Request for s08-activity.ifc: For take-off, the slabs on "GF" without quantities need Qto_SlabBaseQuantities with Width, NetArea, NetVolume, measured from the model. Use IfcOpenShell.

First a look at what the model holds.

```python
import ifcopenshell
import ifcopenshell.util.element
import ifcopenshell.util.unit

model = ifcopenshell.open("s08-activity.ifc")
print(model.schema)
for unit_type in ("LENGTHUNIT", "AREAUNIT", "VOLUMEUNIT"):
    print(unit_type, ifcopenshell.util.unit.calculate_unit_scale(model, unit_type))
storey = next(s for s in model.by_type("IfcBuildingStorey") if s.Name == "GF")
slabs = [e for e in ifcopenshell.util.element.get_decomposition(storey) if e.is_a("IfcSlab")]
for e in sorted(slabs, key=lambda e: e.id()):
    print(e.id(), e.is_a(), e.Name, list(ifcopenshell.util.element.get_psets(e, qtos_only=True)), sep=" | ")
```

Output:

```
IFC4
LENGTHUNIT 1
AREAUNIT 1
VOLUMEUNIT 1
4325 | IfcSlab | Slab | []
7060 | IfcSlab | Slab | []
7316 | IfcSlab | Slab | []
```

```python
import ifcopenshell
import ifcopenshell.api.pset
import ifcopenshell.geom
import ifcopenshell.util.element
import ifcopenshell.util.shape
import ifcopenshell.util.unit

model = ifcopenshell.open("s08-activity.ifc")
unit_scale = ifcopenshell.util.unit.calculate_unit_scale(model)
area_scale = ifcopenshell.util.unit.calculate_unit_scale(model, "AREAUNIT")
volume_scale = ifcopenshell.util.unit.calculate_unit_scale(model, "VOLUMEUNIT")
settings = ifcopenshell.geom.settings()

storey = next(s for s in model.by_type("IfcBuildingStorey") if s.Name == "GF")
slabs = [e for e in ifcopenshell.util.element.get_decomposition(storey) if e.is_a("IfcSlab")]

for e in sorted(slabs, key=lambda e: e.id()):
    if ifcopenshell.util.element.get_psets(e, qtos_only=True, should_inherit=False):
        continue
    # Geometry comes back in metres, in the element's own axes.
    shape = ifcopenshell.geom.create_shape(settings, e)
    values = {
        "Width": ifcopenshell.util.shape.get_z(shape.geometry) / unit_scale,
        "NetArea": ifcopenshell.util.shape.get_footprint_area(shape.geometry) / area_scale,
        "NetVolume": ifcopenshell.util.shape.get_volume(shape.geometry) / volume_scale,
    }
    qto = ifcopenshell.api.pset.add_qto(model, product=e, name="Qto_SlabBaseQuantities")
    ifcopenshell.api.pset.edit_qto(model, qto=qto, properties=values)
    print(e.id(), {k: round(v, 3) for k, v in values.items()})

model.write("s08-activity_updated.ifc")
```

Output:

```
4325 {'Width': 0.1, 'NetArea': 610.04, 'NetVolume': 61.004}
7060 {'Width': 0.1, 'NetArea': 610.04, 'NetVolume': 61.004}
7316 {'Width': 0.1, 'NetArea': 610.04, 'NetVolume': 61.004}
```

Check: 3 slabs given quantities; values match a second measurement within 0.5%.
